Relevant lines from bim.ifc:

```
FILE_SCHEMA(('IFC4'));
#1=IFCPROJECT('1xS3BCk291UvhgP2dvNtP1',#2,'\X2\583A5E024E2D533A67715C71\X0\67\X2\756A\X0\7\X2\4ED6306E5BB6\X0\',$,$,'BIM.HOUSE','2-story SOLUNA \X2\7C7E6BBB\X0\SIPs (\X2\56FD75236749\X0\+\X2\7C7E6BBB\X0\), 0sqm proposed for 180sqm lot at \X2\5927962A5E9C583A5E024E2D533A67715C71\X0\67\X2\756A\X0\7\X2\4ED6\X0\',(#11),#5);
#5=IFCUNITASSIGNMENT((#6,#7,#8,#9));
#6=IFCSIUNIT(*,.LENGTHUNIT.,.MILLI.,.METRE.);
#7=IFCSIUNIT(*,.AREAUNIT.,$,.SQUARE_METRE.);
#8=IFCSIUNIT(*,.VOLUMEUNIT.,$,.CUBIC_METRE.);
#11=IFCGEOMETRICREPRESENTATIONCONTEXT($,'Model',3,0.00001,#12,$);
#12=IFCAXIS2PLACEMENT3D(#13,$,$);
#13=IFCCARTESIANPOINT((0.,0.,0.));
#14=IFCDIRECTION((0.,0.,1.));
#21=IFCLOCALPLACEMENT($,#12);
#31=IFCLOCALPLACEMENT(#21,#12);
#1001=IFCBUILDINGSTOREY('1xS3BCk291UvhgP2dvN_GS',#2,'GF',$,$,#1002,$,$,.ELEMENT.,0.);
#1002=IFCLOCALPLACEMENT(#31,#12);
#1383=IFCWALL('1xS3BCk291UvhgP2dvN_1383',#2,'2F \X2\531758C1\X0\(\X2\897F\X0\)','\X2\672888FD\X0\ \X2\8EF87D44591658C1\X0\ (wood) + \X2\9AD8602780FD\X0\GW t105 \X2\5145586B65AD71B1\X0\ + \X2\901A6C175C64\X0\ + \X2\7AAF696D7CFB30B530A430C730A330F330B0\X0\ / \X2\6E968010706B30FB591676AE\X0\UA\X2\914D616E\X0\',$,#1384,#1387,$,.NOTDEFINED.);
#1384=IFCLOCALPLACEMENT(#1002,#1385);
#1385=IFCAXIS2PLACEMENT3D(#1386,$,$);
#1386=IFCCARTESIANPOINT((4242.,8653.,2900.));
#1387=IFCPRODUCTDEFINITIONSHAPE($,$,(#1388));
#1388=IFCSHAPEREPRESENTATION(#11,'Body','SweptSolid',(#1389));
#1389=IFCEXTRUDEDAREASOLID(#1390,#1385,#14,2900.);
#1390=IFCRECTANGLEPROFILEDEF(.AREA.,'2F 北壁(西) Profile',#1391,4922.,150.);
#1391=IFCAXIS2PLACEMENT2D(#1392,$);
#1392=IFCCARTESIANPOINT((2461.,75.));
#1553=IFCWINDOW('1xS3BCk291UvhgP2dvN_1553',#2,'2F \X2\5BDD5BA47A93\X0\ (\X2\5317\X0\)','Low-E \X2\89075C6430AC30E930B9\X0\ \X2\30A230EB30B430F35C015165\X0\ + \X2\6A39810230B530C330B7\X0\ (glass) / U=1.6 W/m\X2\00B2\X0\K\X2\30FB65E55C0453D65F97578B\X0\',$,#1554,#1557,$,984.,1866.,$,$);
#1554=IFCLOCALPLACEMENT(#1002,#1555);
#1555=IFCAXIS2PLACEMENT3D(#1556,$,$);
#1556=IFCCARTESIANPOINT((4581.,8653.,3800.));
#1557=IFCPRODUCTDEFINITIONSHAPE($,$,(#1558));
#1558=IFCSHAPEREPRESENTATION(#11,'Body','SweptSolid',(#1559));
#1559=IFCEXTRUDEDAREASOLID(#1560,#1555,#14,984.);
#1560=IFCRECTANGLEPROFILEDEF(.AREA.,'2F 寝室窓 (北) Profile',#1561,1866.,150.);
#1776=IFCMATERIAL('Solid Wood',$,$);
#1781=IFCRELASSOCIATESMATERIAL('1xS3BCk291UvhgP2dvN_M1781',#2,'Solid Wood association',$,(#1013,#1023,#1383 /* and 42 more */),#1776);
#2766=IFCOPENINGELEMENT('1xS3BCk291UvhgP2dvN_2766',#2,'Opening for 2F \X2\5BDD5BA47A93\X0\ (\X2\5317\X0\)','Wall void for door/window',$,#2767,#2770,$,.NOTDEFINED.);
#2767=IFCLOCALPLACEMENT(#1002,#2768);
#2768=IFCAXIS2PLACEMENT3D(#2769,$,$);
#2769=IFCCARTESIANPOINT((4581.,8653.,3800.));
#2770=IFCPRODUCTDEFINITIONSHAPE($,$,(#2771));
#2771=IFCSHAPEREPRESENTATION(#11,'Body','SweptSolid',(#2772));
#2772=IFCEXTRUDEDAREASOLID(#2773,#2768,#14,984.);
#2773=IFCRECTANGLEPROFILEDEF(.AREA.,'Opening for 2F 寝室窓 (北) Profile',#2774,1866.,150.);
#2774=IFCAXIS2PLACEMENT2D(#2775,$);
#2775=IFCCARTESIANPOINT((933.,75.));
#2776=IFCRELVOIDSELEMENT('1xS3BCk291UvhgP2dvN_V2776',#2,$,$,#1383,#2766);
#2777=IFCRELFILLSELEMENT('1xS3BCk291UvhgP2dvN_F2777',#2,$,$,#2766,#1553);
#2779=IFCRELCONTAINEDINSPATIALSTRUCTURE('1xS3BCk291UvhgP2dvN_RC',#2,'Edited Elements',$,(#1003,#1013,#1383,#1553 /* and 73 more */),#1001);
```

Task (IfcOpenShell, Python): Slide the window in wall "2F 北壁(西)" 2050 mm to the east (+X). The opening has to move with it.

```python
import ifcopenshell
import ifcopenshell.api.geometry
import ifcopenshell.util.placement
import ifcopenshell.util.unit

model = ifcopenshell.open("bim.ifc")
unit_scale = ifcopenshell.util.unit.calculate_unit_scale(model)

window = model.by_guid("1xS3BCk291UvhgP2dvN_1553")
opening = window.FillsVoids[0].RelatingOpeningElement
wall = opening.VoidsElements[0].RelatingBuildingElement

wall_matrix = ifcopenshell.util.placement.get_local_placement(wall.ObjectPlacement)
shift = wall_matrix[:3, 0] * 2.05 / unit_scale
before = ifcopenshell.util.placement.get_local_placement(window.ObjectPlacement)[:3, 3].copy()

# The window is not placed relative to its opening, so move both.
for product in (opening, window):
    matrix = ifcopenshell.util.placement.get_local_placement(product.ObjectPlacement)
    matrix[:3, 3] += shift
    ifcopenshell.api.geometry.edit_object_placement(model, product=product, matrix=matrix, is_si=False)

after = ifcopenshell.util.placement.get_local_placement(window.ObjectPlacement)[:3, 3]
print("window moved by", (after - before).round(3) + 0.0)

model.write("bim-out.ifc")
```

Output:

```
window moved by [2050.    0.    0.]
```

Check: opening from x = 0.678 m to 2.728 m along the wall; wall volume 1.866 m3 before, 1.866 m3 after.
